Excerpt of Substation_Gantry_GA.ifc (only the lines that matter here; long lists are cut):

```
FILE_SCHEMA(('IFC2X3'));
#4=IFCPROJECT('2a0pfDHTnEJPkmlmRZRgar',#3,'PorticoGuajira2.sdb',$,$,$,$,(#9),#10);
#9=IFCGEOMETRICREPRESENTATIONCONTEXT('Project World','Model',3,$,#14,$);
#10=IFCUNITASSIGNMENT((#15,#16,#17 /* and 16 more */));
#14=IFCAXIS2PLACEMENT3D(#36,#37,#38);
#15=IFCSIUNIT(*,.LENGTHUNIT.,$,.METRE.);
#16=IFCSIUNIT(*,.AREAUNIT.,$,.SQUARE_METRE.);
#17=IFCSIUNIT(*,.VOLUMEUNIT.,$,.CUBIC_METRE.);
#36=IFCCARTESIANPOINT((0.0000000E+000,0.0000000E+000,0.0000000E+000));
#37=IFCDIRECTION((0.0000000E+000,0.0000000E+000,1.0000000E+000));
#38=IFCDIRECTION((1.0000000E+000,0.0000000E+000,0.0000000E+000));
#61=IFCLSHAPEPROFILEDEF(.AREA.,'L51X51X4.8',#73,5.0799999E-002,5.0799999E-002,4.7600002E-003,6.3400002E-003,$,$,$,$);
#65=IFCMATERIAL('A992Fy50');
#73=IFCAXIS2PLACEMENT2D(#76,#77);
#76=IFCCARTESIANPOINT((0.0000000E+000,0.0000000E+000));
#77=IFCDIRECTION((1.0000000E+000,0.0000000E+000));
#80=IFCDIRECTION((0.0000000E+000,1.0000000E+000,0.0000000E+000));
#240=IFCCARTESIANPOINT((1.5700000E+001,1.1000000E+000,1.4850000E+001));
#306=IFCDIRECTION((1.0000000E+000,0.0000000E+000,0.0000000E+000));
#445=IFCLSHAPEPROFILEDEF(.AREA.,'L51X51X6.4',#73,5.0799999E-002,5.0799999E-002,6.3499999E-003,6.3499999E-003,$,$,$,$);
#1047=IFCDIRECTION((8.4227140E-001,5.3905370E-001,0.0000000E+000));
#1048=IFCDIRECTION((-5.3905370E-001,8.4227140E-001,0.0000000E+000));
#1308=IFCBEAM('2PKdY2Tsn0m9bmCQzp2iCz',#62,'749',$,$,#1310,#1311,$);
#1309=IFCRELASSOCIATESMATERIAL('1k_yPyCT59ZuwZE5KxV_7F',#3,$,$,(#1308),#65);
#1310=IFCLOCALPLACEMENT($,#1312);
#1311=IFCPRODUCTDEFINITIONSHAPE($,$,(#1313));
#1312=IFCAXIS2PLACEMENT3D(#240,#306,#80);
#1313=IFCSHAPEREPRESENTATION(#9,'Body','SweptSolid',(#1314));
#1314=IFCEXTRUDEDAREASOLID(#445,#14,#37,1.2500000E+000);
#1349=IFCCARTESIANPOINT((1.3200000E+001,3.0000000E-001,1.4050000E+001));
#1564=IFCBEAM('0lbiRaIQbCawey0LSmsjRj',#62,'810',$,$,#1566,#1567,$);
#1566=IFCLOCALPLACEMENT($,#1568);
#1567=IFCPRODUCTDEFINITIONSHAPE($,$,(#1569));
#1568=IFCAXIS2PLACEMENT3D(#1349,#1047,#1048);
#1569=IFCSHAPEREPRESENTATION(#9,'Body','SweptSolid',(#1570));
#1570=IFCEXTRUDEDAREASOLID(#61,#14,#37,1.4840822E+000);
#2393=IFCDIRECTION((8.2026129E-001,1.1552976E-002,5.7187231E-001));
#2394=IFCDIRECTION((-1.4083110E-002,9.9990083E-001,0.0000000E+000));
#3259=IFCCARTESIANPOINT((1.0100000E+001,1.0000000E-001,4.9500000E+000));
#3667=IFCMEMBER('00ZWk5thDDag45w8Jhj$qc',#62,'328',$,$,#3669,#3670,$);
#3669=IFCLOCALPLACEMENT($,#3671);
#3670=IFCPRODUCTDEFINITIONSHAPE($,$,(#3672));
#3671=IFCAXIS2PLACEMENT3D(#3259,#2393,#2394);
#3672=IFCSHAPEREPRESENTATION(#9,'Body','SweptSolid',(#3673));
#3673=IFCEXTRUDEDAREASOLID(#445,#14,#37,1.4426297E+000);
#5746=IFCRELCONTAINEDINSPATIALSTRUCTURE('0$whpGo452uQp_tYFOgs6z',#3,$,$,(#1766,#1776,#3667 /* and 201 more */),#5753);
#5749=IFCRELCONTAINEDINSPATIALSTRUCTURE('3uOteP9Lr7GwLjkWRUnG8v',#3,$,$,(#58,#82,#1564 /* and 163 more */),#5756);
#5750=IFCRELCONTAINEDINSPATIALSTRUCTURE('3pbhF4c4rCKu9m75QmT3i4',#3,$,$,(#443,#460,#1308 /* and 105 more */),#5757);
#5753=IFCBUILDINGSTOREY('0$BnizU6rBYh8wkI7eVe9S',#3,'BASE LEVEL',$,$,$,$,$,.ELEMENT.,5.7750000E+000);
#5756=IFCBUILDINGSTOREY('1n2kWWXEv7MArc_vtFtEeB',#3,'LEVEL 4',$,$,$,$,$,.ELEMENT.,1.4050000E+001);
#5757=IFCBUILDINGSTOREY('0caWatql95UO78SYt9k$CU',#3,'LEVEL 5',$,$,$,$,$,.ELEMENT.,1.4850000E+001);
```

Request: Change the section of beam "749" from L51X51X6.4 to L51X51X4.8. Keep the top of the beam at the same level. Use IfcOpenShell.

```python
import ifcopenshell
import ifcopenshell.util.element

model = ifcopenshell.open("Substation_Gantry_GA.ifc")

member = model.by_guid("2PKdY2Tsn0m9bmCQzp2iCz")
source = next(p for p in model.by_type("IfcLShapeProfileDef") if p.ProfileName == "L51X51X4.8")

body = next(r for r in member.Representation.Representations if r.RepresentationIdentifier == "Body")
solid = body.Items[0]
old_profile = solid.SweptArea

# Copy the section's sizes but keep this member's own profile position.
profile = ifcopenshell.util.element.copy(model, source)
# Profiles are centred, so shift by half the change in depth to hold the top.
shift = (old_profile.Depth - profile.Depth) / 2
x, y = old_profile.Position.Location.Coordinates
up = (0.0, 1.0)  # upwards, in the solid's own plane
location = model.createIfcCartesianPoint((x + up[0] * shift, y + up[1] * shift))
profile.Position = model.createIfcAxis2Placement2D(location, old_profile.Position.RefDirection)
solid.SweptArea = profile
if not model.get_total_inverses(old_profile):
    ifcopenshell.util.element.remove_deep2(model, old_profile)

print(solid.SweptArea)

model.write("Substation_Gantry_GA_rev.ifc")
```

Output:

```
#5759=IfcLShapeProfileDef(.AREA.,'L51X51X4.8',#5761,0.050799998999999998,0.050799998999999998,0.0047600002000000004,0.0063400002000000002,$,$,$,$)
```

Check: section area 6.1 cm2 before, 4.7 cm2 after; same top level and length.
